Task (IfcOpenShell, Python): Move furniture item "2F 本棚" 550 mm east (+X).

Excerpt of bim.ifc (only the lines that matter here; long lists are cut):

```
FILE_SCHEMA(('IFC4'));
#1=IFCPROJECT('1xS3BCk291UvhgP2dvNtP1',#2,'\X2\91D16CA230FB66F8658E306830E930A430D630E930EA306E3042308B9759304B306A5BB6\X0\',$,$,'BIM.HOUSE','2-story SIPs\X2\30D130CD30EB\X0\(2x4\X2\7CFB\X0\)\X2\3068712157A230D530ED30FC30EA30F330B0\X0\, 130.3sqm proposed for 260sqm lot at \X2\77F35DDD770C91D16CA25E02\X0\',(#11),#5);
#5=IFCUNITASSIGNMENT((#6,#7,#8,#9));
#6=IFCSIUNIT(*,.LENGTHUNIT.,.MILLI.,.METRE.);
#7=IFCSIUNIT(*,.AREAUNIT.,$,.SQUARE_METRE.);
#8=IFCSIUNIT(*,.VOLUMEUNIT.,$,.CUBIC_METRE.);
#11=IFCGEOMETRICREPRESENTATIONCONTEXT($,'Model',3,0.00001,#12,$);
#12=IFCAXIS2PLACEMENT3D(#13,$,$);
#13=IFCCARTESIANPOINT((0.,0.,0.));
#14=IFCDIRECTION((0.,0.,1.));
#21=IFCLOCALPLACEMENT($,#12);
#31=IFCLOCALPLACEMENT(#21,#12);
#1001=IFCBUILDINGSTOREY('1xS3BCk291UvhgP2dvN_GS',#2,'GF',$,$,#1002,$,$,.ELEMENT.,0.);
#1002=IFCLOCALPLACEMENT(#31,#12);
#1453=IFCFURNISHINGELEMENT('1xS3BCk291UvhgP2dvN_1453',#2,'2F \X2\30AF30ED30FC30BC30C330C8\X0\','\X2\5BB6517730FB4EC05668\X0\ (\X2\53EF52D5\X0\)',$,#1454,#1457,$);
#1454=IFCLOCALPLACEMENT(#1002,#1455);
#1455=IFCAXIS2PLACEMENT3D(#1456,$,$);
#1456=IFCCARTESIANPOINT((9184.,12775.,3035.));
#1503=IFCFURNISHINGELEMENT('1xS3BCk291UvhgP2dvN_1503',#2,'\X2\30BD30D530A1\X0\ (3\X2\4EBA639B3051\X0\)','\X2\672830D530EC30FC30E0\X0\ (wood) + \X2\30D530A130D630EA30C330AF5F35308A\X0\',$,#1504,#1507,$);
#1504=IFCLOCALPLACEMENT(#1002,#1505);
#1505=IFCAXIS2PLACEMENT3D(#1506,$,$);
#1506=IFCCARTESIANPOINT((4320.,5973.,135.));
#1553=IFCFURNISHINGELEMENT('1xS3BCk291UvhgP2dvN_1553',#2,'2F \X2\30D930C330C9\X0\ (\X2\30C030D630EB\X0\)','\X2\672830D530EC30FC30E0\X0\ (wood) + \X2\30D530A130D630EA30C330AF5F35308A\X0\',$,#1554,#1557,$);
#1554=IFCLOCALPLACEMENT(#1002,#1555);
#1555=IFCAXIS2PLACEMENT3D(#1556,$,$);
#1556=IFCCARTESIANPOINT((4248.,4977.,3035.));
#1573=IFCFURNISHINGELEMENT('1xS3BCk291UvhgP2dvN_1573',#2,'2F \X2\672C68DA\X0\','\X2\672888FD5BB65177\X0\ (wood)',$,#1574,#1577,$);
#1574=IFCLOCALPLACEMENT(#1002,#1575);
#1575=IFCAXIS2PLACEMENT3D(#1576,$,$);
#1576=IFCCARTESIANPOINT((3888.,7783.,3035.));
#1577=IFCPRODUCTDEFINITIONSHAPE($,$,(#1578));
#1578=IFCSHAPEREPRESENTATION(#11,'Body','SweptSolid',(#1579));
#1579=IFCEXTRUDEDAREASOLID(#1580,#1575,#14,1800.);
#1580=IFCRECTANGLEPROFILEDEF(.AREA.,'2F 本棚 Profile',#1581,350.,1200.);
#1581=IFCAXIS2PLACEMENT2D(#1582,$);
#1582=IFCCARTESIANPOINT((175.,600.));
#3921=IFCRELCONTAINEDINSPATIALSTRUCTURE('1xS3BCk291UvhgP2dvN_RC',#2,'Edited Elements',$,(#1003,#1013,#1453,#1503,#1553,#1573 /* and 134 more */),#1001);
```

```python
import ifcopenshell
import ifcopenshell.api.geometry
import ifcopenshell.util.placement

model = ifcopenshell.open("bim.ifc")

item = model.by_id(1573)
matrix = ifcopenshell.util.placement.get_local_placement(item.ObjectPlacement)
matrix[0, 3] += 550.0
ifcopenshell.api.geometry.edit_object_placement(model, product=item, matrix=matrix, is_si=False)

print(ifcopenshell.util.placement.get_local_placement(item.ObjectPlacement).round(3) + 0.0)

model.write("bim_rev.ifc")
```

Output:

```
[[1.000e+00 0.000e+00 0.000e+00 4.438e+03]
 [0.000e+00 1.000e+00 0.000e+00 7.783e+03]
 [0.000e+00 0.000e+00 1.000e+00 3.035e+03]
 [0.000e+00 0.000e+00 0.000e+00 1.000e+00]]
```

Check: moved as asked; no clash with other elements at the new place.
